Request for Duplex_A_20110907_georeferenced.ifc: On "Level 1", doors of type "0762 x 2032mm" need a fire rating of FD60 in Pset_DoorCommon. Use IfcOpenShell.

First a look at what the model holds.

```python
import ifcopenshell
import ifcopenshell.util.element

model = ifcopenshell.open("Duplex_A_20110907_georeferenced.ifc")
print(model.schema)
storey = next(s for s in model.by_type("IfcBuildingStorey") if s.Name == "Level 1")
doors = [e for e in ifcopenshell.util.element.get_decomposition(storey) if e.is_a("IfcDoor")]
seen = {}
for e in doors:
    element_type = ifcopenshell.util.element.get_type(e)
    key = (element_type.Name if element_type != e and element_type else None, ifcopenshell.util.element.get_pset(e, "Pset_DoorCommon", "FireRating"))
    seen[key] = seen.get(key, 0) + 1
for (name, value), count in sorted(seen.items(), key=str):
    print(count, "x", name, "|", value)
```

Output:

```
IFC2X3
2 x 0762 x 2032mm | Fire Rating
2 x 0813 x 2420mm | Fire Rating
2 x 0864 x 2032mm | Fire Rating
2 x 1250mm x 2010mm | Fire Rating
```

```python
import ifcopenshell
import ifcopenshell.api.pset
import ifcopenshell.util.element

model = ifcopenshell.open("Duplex_A_20110907_georeferenced.ifc")

storey = next(s for s in model.by_type("IfcBuildingStorey") if s.Name == "Level 1")
doors = [e for e in ifcopenshell.util.element.get_decomposition(storey) if e.is_a("IfcDoor")]

count = 0
for e in doors:
    element_type = ifcopenshell.util.element.get_type(e)
    if element_type in (None, e) or element_type.Name != "0762 x 2032mm":
        continue
    # add_pset returns the element's existing set when there is one.
    pset = ifcopenshell.api.pset.add_pset(model, product=e, name="Pset_DoorCommon")
    ifcopenshell.api.pset.edit_pset(model, pset=pset, properties={"FireRating": "FD60"})
    count += 1

print(count, "doors updated")

model.write("Duplex_A_20110907_georeferenced_rev.ifc")
```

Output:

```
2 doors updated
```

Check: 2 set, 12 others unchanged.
